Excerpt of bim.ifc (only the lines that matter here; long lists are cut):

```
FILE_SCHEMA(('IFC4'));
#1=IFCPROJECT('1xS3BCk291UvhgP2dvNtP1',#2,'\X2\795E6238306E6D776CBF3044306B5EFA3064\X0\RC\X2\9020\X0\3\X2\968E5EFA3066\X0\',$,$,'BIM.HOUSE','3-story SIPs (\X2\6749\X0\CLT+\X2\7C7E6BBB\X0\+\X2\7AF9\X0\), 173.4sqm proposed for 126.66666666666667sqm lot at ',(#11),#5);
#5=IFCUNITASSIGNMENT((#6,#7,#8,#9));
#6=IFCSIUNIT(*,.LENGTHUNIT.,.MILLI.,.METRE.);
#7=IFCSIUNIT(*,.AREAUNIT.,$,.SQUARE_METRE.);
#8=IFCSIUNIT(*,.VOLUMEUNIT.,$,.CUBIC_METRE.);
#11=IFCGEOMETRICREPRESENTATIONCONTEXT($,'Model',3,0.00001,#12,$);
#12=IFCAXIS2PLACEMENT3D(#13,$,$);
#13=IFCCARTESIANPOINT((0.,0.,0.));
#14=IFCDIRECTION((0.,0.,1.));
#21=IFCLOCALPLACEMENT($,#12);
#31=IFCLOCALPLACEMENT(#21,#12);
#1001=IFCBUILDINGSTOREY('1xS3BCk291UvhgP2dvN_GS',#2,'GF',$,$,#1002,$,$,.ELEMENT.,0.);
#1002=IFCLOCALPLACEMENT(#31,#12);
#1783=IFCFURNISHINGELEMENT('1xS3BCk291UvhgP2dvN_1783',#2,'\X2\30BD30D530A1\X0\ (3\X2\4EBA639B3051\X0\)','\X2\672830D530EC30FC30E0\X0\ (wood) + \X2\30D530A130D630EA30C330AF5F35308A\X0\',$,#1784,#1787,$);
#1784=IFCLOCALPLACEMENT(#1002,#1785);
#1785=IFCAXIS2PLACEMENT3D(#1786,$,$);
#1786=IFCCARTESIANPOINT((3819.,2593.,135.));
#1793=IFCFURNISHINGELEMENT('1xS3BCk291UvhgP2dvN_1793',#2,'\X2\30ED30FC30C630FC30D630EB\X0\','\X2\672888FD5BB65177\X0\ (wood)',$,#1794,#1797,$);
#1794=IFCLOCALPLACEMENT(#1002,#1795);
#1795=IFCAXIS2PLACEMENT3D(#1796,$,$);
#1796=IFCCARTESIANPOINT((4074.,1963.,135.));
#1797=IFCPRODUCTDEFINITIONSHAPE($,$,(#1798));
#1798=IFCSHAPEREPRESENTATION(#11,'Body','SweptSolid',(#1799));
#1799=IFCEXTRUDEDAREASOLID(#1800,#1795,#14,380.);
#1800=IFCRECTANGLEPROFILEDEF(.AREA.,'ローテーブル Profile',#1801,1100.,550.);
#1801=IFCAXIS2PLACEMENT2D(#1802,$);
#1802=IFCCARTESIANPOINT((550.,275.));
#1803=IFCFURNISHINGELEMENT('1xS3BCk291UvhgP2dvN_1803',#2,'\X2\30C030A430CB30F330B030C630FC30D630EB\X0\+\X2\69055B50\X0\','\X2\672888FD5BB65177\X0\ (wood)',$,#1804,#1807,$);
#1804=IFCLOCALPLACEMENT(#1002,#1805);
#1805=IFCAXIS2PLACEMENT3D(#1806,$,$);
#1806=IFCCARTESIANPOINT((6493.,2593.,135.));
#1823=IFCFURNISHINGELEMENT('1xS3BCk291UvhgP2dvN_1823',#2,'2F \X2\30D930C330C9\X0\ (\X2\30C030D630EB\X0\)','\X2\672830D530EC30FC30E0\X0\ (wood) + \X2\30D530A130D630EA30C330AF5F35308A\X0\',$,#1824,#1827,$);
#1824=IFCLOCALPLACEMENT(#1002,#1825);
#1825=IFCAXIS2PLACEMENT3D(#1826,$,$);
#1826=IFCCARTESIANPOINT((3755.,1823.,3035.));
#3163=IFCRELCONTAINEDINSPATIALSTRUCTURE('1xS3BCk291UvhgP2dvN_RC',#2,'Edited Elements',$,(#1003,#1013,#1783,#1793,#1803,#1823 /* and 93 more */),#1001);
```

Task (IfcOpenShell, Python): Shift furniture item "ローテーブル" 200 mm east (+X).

```python
import ifcopenshell
import ifcopenshell.api.geometry
import ifcopenshell.util.placement
import ifcopenshell.util.unit

model = ifcopenshell.open("bim.ifc")
unit_scale = ifcopenshell.util.unit.calculate_unit_scale(model)

item = model.by_id(1793)
matrix = ifcopenshell.util.placement.get_local_placement(item.ObjectPlacement)
matrix[0, 3] += 0.2 / unit_scale
ifcopenshell.api.geometry.edit_object_placement(model, product=item, matrix=matrix, is_si=False)

print(ifcopenshell.util.placement.get_local_placement(item.ObjectPlacement).round(3) + 0.0)

model.write("bim-out.ifc")
```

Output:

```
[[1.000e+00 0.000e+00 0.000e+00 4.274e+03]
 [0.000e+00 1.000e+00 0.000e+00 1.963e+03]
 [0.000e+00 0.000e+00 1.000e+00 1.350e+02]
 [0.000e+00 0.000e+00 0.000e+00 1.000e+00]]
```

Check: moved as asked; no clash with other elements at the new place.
